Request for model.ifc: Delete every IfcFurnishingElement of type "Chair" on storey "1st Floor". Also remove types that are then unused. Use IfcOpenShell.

First a look at what the model holds.

```python
import ifcopenshell
import ifcopenshell.util.element

model = ifcopenshell.open("model.ifc")
print(model.schema)
storey = next(s for s in model.by_type("IfcBuildingStorey") if s.Name == "1st Floor")
furniture = [e for e in ifcopenshell.util.element.get_decomposition(storey) if e.is_a("IfcFurnishingElement")]
seen = {}
for e in furniture:
    element_type = ifcopenshell.util.element.get_type(e)
    name = element_type.Name if element_type not in (None, e) else None
    seen[name] = seen.get(name, 0) + 1
for name, count in sorted(seen.items(), key=str):
    print(count, "x", name)
```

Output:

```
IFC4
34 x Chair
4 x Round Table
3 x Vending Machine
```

```python
import ifcopenshell
import ifcopenshell.api.root
import ifcopenshell.util.element

model = ifcopenshell.open("model.ifc")

storey = next(s for s in model.by_type("IfcBuildingStorey") if s.Name == "1st Floor")
furniture = [e for e in ifcopenshell.util.element.get_decomposition(storey) if e.is_a("IfcFurnishingElement")]
targets = [e for e in furniture if (t := ifcopenshell.util.element.get_type(e)) not in (None, e) and t.Name == "Chair"]
types = {ifcopenshell.util.element.get_type(e) for e in targets} - {None, *targets}

for e in targets:
    ifcopenshell.api.root.remove_product(model, product=e)
print(len(targets), "removed")

unused = [t for t in types if not ifcopenshell.util.element.get_types(t)]
for t in unused:
    ifcopenshell.api.root.remove_product(model, product=t)
print(len(unused), "unused types removed")

model.write("model_rev.ifc")
```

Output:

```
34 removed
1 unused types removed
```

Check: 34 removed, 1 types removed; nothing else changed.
